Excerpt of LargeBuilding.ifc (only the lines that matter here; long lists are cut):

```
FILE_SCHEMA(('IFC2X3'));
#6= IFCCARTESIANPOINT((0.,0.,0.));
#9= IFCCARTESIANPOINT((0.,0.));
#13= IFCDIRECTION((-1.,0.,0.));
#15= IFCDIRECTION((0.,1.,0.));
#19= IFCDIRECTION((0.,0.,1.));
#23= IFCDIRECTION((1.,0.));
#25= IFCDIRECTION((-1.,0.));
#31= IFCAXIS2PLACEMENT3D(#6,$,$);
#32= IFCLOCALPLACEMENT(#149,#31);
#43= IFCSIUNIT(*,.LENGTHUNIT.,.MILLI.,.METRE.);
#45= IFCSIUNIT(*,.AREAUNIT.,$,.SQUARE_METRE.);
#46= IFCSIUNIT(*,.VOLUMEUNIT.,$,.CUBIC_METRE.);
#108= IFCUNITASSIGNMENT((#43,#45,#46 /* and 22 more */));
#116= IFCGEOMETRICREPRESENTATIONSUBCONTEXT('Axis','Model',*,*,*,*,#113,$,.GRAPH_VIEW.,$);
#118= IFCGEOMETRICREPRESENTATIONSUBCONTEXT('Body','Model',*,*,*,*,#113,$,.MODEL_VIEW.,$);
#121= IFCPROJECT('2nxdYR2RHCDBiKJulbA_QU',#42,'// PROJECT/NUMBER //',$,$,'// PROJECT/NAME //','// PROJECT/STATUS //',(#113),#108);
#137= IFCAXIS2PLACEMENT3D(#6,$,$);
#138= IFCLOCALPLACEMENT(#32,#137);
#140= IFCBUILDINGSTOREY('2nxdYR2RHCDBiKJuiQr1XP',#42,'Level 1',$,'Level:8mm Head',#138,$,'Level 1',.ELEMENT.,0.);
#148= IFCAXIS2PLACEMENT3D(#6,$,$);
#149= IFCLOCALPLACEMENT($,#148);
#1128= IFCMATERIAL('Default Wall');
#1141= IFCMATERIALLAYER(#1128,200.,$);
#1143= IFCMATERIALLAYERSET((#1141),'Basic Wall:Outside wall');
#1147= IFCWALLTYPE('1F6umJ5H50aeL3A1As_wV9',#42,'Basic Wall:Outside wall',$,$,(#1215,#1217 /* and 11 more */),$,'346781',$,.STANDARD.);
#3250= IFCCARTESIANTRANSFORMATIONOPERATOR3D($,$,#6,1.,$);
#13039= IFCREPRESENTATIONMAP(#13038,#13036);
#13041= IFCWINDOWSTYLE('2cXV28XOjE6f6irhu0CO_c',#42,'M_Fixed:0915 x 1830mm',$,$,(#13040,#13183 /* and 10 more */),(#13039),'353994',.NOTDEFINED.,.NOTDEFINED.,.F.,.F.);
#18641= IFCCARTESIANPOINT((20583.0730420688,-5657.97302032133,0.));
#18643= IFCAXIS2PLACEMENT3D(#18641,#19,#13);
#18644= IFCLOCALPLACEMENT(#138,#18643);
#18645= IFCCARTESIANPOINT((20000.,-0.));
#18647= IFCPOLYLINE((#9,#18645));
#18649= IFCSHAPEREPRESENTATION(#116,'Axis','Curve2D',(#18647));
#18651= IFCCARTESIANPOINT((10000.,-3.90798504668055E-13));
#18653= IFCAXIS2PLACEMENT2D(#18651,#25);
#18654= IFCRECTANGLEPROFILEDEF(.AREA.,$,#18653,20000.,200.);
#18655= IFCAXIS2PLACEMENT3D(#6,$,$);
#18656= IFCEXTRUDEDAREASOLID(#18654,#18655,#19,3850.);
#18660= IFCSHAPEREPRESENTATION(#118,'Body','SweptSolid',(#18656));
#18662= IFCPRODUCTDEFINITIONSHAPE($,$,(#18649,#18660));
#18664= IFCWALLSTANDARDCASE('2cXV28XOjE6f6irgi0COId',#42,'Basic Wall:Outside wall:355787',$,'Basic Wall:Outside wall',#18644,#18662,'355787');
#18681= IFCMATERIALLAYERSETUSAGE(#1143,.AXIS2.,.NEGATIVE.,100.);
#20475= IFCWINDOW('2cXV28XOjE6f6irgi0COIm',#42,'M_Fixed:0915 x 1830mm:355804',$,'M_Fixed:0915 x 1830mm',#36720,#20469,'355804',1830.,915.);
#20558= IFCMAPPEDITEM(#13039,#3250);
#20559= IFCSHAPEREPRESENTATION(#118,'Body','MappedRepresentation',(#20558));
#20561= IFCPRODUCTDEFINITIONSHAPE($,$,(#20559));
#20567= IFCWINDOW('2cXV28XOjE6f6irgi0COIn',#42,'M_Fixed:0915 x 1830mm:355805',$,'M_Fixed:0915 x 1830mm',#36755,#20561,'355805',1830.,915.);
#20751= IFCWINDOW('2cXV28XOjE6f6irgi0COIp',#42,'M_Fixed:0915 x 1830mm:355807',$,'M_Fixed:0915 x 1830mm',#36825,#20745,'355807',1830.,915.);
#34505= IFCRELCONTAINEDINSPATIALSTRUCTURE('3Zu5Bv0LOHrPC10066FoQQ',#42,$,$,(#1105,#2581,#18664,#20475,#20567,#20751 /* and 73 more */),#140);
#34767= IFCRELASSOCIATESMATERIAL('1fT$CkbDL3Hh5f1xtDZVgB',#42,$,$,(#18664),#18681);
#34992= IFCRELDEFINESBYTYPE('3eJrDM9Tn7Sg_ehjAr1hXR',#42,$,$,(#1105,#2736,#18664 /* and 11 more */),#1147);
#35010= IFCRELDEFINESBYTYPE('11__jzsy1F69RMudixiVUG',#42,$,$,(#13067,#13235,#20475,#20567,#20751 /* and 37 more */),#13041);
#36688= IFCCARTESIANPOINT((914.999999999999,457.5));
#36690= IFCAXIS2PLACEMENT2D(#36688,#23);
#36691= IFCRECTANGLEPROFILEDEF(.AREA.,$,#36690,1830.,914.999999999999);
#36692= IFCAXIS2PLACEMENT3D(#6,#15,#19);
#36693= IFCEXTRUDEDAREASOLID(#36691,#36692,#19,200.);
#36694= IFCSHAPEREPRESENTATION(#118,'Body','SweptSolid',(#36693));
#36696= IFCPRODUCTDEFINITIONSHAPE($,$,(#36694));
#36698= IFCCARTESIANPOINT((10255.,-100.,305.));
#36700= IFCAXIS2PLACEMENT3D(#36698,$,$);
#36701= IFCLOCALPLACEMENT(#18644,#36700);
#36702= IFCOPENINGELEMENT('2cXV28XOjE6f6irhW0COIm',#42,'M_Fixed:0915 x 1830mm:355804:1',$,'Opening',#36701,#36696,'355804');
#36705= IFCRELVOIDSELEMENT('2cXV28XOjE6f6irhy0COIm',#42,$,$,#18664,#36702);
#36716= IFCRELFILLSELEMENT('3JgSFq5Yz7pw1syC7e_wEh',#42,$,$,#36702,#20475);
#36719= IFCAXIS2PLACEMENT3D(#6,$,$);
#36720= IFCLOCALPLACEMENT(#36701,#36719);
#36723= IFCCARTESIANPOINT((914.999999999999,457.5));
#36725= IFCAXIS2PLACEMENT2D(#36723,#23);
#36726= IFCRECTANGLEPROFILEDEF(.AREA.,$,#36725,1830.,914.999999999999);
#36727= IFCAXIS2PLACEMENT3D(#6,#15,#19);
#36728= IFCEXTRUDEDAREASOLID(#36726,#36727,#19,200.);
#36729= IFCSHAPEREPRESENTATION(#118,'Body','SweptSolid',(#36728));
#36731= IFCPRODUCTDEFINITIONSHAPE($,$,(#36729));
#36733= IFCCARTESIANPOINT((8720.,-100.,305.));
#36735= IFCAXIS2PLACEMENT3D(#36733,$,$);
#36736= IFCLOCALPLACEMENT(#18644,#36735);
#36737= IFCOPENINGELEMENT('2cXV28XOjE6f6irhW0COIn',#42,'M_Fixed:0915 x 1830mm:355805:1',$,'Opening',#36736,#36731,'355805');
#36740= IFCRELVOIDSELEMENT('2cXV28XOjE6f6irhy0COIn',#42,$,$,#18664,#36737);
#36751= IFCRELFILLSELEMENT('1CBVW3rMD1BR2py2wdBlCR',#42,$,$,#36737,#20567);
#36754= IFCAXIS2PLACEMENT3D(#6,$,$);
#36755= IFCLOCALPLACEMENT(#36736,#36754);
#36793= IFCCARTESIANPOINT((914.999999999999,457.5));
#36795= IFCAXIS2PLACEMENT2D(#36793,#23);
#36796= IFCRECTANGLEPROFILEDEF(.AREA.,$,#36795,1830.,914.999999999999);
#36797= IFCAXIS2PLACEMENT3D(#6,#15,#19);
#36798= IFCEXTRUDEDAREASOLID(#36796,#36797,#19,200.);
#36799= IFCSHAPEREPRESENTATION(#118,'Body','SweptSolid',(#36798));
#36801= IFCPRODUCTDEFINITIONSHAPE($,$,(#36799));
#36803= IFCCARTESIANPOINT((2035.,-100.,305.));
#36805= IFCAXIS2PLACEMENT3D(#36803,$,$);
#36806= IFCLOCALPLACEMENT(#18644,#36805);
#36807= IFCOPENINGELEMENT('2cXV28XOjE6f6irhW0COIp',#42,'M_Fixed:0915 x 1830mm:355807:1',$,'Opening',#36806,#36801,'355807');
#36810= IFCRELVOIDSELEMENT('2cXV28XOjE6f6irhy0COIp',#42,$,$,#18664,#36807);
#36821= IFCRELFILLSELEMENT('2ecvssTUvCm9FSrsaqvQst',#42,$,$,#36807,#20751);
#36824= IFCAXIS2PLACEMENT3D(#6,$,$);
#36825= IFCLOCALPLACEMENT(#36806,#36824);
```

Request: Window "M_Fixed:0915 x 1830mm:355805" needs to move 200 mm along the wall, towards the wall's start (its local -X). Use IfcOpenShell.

```python
import ifcopenshell
import ifcopenshell.api.geometry
import ifcopenshell.util.placement
import ifcopenshell.util.unit

model = ifcopenshell.open("LargeBuilding.ifc")
unit_scale = ifcopenshell.util.unit.calculate_unit_scale(model)

window = model.by_guid("2cXV28XOjE6f6irgi0COIn")
opening = window.FillsVoids[0].RelatingOpeningElement
wall = opening.VoidsElements[0].RelatingBuildingElement

wall_matrix = ifcopenshell.util.placement.get_local_placement(wall.ObjectPlacement)
shift = wall_matrix[:3, 0] * -0.2 / unit_scale
before = ifcopenshell.util.placement.get_local_placement(window.ObjectPlacement)[:3, 3].copy()

# The window is placed relative to its opening, so it follows when the opening moves.
matrix = ifcopenshell.util.placement.get_local_placement(opening.ObjectPlacement)
matrix[:3, 3] += shift
ifcopenshell.api.geometry.edit_object_placement(
    model, product=opening, matrix=matrix, is_si=False, should_transform_children=True
)

after = ifcopenshell.util.placement.get_local_placement(window.ObjectPlacement)[:3, 3]
print("window moved by", (after - before).round(3) + 0.0)

model.write("LargeBuilding_v2.ifc")
```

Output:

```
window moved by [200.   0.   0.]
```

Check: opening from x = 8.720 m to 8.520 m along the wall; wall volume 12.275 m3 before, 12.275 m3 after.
